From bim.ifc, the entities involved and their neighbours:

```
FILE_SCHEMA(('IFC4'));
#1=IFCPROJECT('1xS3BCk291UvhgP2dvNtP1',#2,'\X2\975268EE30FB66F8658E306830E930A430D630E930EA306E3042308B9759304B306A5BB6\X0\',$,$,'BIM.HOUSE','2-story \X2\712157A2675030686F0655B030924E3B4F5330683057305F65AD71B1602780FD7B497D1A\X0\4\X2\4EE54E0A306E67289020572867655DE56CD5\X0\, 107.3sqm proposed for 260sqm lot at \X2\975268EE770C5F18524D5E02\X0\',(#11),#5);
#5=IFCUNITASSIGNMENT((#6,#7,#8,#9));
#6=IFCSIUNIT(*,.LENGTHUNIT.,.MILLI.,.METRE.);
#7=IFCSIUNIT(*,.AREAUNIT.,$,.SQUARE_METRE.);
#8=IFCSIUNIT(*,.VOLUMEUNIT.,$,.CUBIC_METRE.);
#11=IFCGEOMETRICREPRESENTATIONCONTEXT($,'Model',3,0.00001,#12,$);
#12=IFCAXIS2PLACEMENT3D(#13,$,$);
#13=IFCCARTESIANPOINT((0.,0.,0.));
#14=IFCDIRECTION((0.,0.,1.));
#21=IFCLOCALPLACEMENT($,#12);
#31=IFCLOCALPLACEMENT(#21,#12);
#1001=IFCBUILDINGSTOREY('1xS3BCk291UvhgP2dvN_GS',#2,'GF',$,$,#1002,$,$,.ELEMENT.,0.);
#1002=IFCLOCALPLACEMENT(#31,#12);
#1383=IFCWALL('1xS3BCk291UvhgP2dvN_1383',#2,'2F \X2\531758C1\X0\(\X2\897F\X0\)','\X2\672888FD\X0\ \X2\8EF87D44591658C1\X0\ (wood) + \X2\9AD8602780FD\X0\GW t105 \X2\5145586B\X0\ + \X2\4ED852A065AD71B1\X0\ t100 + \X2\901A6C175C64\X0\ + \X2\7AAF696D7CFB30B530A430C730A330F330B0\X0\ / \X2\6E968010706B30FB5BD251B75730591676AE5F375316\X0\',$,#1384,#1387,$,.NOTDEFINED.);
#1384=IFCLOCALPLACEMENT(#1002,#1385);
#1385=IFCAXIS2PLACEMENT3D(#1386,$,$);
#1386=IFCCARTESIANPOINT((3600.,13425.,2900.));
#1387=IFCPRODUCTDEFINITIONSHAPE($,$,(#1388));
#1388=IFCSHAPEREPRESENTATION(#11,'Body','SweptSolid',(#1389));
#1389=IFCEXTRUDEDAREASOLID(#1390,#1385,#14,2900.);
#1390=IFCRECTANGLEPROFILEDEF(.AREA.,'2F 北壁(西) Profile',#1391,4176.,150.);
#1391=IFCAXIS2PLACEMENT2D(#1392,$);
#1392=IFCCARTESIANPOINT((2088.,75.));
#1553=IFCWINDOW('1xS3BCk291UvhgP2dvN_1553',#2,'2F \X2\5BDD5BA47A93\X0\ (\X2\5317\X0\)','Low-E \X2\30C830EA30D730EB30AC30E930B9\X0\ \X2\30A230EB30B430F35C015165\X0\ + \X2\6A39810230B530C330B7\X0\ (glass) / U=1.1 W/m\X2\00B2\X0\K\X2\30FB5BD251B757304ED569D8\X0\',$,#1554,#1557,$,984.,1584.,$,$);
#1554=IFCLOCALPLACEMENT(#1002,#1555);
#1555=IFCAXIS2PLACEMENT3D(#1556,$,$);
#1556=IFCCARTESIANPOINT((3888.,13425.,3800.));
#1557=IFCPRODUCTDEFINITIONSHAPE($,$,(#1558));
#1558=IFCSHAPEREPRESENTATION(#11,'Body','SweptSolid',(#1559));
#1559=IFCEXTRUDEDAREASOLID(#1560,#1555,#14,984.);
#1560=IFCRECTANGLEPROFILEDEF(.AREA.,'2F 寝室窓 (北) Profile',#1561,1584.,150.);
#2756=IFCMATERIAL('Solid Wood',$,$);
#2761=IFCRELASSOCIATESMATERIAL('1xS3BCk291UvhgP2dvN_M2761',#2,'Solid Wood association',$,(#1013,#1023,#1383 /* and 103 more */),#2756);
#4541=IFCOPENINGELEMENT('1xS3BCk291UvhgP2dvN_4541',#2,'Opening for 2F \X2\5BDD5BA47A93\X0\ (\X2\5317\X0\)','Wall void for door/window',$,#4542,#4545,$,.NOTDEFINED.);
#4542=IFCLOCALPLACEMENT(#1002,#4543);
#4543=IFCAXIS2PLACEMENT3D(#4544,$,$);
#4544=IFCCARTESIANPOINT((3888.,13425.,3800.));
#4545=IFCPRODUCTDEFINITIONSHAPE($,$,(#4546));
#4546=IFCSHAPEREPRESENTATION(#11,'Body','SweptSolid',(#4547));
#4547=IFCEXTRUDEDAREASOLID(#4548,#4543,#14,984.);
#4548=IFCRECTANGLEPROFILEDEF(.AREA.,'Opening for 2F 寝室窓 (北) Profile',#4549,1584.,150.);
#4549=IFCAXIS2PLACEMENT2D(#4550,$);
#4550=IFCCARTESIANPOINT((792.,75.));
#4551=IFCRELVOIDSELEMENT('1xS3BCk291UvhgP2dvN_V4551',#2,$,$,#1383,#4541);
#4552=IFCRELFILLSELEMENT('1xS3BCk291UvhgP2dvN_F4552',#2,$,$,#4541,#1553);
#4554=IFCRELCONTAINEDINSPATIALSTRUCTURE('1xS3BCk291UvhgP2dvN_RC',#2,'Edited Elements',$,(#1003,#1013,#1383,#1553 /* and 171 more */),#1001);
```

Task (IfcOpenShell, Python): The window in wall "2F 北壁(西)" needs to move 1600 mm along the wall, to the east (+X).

```python
import ifcopenshell
import ifcopenshell.api.geometry
import ifcopenshell.util.placement

model = ifcopenshell.open("bim.ifc")

window = model.by_guid("1xS3BCk291UvhgP2dvN_1553")
opening = window.FillsVoids[0].RelatingOpeningElement
wall = opening.VoidsElements[0].RelatingBuildingElement

wall_matrix = ifcopenshell.util.placement.get_local_placement(wall.ObjectPlacement)
shift = wall_matrix[:3, 0] * 1600.0
before = ifcopenshell.util.placement.get_local_placement(window.ObjectPlacement)[:3, 3].copy()

# The window is not placed relative to its opening, so move both.
for product in (opening, window):
    matrix = ifcopenshell.util.placement.get_local_placement(product.ObjectPlacement)
    matrix[:3, 3] += shift
    ifcopenshell.api.geometry.edit_object_placement(model, product=product, matrix=matrix, is_si=False)

after = ifcopenshell.util.placement.get_local_placement(window.ObjectPlacement)[:3, 3]
print("window moved by", (after - before).round(3) + 0.0)

model.write("bim_updated.ifc")
```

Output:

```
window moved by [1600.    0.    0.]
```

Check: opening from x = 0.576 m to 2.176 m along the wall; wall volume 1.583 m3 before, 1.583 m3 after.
